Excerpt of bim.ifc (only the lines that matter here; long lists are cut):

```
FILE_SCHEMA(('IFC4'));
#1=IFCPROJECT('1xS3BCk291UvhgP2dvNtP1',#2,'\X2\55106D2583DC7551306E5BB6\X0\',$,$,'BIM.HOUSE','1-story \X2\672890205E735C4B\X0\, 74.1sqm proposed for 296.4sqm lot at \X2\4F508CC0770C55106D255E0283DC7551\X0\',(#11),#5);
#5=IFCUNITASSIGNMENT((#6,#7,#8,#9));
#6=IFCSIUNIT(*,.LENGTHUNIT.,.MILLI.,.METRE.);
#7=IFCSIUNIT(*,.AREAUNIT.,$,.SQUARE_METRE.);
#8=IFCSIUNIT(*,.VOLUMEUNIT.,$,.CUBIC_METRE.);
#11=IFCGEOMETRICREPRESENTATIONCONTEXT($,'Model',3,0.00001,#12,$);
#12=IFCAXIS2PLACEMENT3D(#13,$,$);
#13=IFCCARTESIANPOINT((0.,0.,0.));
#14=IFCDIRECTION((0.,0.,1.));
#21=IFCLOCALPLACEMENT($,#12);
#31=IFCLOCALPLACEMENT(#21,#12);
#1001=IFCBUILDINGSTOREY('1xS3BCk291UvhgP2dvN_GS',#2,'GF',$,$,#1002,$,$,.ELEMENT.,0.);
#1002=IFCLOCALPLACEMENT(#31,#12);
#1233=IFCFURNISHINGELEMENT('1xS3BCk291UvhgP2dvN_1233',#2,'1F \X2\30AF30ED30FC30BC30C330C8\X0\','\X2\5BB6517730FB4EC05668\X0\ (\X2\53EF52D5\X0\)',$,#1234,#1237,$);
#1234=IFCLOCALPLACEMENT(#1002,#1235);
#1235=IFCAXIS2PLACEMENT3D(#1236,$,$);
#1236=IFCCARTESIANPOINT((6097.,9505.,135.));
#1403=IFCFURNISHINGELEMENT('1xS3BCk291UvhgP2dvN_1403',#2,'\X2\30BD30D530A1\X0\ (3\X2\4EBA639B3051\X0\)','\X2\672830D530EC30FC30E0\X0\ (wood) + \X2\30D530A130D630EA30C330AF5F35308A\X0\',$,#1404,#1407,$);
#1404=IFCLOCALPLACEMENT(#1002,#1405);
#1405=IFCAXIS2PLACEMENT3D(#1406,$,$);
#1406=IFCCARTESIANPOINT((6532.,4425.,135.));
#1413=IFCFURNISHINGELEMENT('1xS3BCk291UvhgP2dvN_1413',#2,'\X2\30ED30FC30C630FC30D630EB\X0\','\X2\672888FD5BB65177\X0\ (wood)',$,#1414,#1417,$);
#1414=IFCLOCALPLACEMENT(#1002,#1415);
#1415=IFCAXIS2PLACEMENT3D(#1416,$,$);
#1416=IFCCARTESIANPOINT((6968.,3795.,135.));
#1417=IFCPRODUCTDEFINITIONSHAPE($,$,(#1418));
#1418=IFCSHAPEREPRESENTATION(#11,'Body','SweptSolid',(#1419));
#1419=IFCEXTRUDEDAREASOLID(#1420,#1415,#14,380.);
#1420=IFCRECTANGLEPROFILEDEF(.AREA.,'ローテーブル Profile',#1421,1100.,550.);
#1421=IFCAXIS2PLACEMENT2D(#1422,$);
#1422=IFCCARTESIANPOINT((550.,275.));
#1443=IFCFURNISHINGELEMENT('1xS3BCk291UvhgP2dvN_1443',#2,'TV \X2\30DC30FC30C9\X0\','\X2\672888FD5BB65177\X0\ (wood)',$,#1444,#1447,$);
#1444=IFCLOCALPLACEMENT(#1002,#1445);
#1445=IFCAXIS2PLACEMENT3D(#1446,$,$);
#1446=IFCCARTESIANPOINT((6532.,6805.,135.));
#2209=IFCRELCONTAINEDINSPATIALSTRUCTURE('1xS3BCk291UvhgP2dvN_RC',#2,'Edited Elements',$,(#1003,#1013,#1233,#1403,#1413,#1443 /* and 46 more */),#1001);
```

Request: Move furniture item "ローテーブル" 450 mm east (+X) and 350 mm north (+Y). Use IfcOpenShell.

```python
import ifcopenshell
import ifcopenshell.api.geometry
import ifcopenshell.util.placement
import ifcopenshell.util.unit

model = ifcopenshell.open("bim.ifc")
unit_scale = ifcopenshell.util.unit.calculate_unit_scale(model)

item = model.by_guid("1xS3BCk291UvhgP2dvN_1413")
matrix = ifcopenshell.util.placement.get_local_placement(item.ObjectPlacement)
matrix[0, 3] += 0.45 / unit_scale
matrix[1, 3] += 0.35 / unit_scale
ifcopenshell.api.geometry.edit_object_placement(model, product=item, matrix=matrix, is_si=False)

print(ifcopenshell.util.placement.get_local_placement(item.ObjectPlacement).round(3) + 0.0)

model.write("bim_rev.ifc")
```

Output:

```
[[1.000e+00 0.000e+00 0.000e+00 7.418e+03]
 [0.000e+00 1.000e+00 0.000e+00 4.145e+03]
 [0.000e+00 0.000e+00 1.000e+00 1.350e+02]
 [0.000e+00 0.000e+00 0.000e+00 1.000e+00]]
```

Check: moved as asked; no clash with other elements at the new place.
